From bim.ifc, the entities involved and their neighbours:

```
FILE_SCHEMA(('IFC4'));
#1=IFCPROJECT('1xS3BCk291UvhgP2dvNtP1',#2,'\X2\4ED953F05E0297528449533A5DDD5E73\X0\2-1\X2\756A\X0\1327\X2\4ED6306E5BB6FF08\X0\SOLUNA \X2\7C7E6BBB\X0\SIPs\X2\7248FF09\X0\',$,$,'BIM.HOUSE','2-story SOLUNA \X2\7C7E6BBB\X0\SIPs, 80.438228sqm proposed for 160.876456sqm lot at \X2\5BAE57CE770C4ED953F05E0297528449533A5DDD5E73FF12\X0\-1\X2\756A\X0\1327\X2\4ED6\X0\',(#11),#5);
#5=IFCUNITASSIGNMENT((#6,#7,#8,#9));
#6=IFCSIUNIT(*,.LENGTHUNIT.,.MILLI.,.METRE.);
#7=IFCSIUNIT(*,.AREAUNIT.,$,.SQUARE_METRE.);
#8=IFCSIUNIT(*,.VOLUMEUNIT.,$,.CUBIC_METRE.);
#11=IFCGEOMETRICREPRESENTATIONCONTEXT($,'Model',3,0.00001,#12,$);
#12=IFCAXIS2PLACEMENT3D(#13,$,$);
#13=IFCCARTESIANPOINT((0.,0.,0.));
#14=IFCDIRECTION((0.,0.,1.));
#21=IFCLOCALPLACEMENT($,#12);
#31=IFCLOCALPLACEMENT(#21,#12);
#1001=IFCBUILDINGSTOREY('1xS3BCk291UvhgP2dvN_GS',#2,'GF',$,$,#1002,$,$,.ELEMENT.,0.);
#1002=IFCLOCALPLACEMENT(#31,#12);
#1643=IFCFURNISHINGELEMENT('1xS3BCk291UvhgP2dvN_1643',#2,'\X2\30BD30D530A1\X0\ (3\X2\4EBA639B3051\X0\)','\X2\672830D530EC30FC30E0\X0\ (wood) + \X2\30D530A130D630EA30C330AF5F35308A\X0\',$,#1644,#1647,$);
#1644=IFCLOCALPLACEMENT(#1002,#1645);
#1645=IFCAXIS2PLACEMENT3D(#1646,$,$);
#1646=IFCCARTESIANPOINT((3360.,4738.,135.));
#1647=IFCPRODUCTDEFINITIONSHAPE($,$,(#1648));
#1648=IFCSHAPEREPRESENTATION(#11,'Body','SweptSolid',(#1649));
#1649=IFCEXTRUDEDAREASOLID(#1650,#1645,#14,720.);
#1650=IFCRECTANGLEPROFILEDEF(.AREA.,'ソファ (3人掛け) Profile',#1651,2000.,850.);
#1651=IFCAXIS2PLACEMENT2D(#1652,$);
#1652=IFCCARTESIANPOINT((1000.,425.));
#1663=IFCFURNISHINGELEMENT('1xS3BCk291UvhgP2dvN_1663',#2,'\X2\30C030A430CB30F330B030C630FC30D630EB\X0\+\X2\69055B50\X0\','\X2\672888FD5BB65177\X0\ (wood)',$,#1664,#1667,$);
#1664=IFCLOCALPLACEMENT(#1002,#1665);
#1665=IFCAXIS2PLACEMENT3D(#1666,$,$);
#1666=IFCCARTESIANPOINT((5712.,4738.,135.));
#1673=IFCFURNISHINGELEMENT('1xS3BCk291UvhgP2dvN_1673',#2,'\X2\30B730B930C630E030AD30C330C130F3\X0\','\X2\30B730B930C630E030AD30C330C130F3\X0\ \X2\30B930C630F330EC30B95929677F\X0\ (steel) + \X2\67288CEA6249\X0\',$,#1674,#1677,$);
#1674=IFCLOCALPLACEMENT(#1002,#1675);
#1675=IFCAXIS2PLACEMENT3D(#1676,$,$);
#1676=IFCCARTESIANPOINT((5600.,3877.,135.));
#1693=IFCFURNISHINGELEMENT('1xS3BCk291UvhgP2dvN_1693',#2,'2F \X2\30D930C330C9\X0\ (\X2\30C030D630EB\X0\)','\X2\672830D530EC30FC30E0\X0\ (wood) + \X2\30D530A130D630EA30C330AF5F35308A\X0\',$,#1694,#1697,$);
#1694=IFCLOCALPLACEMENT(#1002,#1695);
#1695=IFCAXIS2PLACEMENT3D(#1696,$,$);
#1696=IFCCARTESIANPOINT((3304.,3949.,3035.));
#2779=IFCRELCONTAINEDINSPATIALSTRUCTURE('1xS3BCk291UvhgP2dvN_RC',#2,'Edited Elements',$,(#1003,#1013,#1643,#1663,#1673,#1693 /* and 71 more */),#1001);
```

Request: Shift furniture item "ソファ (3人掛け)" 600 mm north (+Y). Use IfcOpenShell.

```python
import ifcopenshell
import ifcopenshell.api.geometry
import ifcopenshell.util.placement
import ifcopenshell.util.unit

model = ifcopenshell.open("bim.ifc")
unit_scale = ifcopenshell.util.unit.calculate_unit_scale(model)

item = model.by_guid("1xS3BCk291UvhgP2dvN_1643")
matrix = ifcopenshell.util.placement.get_local_placement(item.ObjectPlacement)
matrix[1, 3] += 0.6 / unit_scale
ifcopenshell.api.geometry.edit_object_placement(model, product=item, matrix=matrix, is_si=False)

print(ifcopenshell.util.placement.get_local_placement(item.ObjectPlacement).round(3) + 0.0)

model.write("bim_rev.ifc")
```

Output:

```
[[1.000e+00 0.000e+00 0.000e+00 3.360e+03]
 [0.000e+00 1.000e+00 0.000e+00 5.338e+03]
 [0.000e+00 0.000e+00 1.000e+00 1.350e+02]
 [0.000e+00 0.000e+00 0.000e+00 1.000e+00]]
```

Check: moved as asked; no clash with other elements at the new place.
